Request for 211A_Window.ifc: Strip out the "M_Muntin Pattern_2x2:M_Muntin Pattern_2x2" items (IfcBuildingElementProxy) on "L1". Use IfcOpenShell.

First a look at what the model holds.

```python
import ifcopenshell
import ifcopenshell.util.element

model = ifcopenshell.open("211A_Window.ifc")
print(model.schema)
storey = next(s for s in model.by_type("IfcBuildingStorey") if s.Name == "L1")
proxies = [e for e in ifcopenshell.util.element.get_decomposition(storey) if e.is_a("IfcBuildingElementProxy")]
seen = {}
for e in proxies:
    element_type = ifcopenshell.util.element.get_type(e)
    name = element_type.Name if element_type not in (None, e) else None
    seen[name] = seen.get(name, 0) + 1
for name, count in sorted(seen.items(), key=str):
    print(count, "x", name)
```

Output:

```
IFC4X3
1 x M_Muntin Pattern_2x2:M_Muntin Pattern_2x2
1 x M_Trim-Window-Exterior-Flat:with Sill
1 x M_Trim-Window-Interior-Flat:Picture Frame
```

```python
import ifcopenshell
import ifcopenshell.api.root
import ifcopenshell.util.element

model = ifcopenshell.open("211A_Window.ifc")

storey = next(s for s in model.by_type("IfcBuildingStorey") if s.Name == "L1")
proxies = [e for e in ifcopenshell.util.element.get_decomposition(storey) if e.is_a("IfcBuildingElementProxy")]
targets = [e for e in proxies if (t := ifcopenshell.util.element.get_type(e)) not in (None, e) and t.Name == "M_Muntin Pattern_2x2:M_Muntin Pattern_2x2"]

for e in targets:
    ifcopenshell.api.root.remove_product(model, product=e)
print(len(targets), "removed")

model.write("211A_Window_updated.ifc")
```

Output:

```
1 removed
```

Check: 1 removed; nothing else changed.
